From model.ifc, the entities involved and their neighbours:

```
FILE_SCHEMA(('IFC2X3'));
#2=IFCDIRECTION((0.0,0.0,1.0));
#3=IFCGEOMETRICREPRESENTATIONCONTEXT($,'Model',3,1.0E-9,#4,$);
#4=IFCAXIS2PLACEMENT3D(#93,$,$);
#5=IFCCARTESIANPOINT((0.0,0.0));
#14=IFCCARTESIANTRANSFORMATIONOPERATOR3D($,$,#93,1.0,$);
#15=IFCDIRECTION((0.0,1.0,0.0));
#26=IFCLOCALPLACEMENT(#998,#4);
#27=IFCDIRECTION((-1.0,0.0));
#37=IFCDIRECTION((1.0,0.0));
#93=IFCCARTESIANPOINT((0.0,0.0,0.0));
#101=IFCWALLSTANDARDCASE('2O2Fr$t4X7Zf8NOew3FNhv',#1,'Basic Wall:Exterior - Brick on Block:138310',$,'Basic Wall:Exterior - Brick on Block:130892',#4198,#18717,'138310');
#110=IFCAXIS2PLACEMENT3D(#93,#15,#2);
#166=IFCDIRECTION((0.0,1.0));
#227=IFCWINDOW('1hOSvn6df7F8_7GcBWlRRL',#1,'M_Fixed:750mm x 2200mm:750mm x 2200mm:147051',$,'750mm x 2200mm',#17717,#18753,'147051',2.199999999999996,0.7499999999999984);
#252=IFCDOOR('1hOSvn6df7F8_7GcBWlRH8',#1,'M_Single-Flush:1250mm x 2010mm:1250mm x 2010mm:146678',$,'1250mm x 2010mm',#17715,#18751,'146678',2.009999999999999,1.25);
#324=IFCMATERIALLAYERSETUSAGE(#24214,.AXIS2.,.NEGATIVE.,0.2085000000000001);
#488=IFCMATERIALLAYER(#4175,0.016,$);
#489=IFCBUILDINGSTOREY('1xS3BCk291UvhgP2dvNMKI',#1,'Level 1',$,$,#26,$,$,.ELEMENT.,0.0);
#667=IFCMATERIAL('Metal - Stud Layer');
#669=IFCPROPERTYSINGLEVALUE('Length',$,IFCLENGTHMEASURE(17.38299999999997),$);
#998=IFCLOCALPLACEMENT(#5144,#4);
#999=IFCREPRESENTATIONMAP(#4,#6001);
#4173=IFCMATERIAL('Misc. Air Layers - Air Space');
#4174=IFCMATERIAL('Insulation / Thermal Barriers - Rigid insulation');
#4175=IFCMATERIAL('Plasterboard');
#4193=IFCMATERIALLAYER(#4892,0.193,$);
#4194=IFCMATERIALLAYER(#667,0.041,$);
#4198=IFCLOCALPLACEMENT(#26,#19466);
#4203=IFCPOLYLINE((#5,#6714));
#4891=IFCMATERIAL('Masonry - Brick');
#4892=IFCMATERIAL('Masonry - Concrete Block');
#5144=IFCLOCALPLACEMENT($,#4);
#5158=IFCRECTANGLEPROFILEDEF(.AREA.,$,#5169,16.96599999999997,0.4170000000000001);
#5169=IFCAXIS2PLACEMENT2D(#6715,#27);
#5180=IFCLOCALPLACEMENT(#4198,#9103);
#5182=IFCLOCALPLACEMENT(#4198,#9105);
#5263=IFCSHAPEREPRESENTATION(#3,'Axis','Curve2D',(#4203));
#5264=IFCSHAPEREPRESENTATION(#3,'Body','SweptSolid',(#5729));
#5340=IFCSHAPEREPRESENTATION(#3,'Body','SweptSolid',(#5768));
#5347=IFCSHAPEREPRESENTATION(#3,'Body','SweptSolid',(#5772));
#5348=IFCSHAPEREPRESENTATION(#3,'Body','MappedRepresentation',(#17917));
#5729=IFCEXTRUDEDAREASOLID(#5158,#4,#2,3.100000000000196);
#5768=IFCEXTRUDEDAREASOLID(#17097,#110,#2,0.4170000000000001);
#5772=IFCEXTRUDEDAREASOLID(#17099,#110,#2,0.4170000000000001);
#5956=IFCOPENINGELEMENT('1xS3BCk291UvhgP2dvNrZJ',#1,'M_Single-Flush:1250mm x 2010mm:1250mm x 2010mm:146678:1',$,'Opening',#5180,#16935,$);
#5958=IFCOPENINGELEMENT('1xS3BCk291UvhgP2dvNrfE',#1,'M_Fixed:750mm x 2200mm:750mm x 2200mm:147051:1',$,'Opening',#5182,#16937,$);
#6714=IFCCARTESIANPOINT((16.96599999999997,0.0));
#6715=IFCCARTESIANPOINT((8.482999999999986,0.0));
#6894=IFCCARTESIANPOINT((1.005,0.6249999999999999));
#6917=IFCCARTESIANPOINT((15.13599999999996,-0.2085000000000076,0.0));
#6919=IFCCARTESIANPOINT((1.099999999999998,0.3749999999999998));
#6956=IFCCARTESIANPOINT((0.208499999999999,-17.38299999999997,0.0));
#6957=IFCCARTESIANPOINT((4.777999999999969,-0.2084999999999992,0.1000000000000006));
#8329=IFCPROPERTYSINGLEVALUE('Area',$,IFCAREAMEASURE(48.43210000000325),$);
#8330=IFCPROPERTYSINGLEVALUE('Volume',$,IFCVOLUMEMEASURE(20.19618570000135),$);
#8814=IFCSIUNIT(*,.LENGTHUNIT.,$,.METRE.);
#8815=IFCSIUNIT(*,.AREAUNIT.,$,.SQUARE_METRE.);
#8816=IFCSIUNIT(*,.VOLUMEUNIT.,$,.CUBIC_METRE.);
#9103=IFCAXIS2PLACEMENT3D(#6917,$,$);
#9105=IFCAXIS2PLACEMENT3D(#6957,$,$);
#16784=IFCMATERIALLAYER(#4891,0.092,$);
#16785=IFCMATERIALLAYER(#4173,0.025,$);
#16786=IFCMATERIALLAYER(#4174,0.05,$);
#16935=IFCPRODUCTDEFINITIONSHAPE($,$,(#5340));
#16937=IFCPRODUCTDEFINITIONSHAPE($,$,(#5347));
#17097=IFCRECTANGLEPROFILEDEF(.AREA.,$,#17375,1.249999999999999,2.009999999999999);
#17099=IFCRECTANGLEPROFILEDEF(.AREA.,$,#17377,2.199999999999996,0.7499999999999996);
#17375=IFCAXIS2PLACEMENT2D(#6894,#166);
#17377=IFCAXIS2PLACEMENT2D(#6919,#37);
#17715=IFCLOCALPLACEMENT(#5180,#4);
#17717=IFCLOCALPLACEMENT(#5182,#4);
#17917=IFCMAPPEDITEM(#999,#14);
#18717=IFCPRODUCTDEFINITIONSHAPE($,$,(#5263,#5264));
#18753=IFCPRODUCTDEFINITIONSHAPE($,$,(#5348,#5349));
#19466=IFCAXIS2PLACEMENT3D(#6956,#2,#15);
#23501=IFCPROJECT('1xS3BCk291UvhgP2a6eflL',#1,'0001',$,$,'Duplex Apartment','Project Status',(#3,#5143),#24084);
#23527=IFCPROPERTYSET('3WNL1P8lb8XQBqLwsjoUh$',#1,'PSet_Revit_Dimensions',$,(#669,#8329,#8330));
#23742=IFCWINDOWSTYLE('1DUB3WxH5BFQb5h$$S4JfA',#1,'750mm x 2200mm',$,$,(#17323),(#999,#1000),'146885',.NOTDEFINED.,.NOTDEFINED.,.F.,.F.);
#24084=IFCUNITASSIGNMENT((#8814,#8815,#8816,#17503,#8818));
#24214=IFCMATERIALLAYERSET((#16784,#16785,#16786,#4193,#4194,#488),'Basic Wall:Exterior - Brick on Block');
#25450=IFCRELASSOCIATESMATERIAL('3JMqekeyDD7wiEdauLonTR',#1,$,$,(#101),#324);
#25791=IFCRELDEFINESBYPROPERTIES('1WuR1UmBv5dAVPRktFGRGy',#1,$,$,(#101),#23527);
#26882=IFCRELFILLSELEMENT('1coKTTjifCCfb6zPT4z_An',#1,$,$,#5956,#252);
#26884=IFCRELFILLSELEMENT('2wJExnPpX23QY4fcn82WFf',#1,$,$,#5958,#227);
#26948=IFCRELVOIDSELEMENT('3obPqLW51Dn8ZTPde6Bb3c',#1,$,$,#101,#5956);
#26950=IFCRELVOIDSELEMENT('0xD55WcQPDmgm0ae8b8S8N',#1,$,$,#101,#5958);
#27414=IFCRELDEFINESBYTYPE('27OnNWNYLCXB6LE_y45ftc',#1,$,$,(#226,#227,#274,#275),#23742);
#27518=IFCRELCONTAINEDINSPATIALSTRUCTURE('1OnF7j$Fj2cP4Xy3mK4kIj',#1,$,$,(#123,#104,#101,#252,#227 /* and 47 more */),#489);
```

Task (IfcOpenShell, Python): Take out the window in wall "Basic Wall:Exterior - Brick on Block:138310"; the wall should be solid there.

```python
import ifcopenshell
import ifcopenshell.api.feature
import ifcopenshell.api.pset
import ifcopenshell.api.root
import ifcopenshell.geom
import ifcopenshell.util.element
import ifcopenshell.util.shape
import ifcopenshell.util.unit

model = ifcopenshell.open("model.ifc")
area_scale = ifcopenshell.util.unit.calculate_unit_scale(model, "AREAUNIT")
volume_scale = ifcopenshell.util.unit.calculate_unit_scale(model, "VOLUMEUNIT")
settings = ifcopenshell.geom.settings()


def volume(element):
    """Net volume in cubic metres, openings subtracted."""
    shape = ifcopenshell.geom.create_shape(settings, element)
    return ifcopenshell.util.shape.get_volume(shape.geometry)


window = model.by_guid("1hOSvn6df7F8_7GcBWlRRL")
opening = window.FillsVoids[0].RelatingOpeningElement
wall = opening.VoidsElements[0].RelatingBuildingElement
before = volume(wall)

ifcopenshell.api.root.remove_product(model, product=window)
ifcopenshell.api.feature.remove_feature(model, feature=opening)

after = volume(wall)
thickness = 0.417  # wall thickness in metres

# Update the wall's stored quantities.
pset = model.by_id(ifcopenshell.util.element.get_pset(wall, "PSet_Revit_Dimensions", should_inherit=False)["id"])
ifcopenshell.api.pset.edit_pset(model, pset=pset, properties={
    "Area": model.create_entity("IfcAreaMeasure", after / thickness / area_scale),
    "Volume": model.create_entity("IfcVolumeMeasure", after / volume_scale),
})

print(f"wall volume {before:.3f} -> {after:.3f} m3")

model.write("model_v2.ifc")
```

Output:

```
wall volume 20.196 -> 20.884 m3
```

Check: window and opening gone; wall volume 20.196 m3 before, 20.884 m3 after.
